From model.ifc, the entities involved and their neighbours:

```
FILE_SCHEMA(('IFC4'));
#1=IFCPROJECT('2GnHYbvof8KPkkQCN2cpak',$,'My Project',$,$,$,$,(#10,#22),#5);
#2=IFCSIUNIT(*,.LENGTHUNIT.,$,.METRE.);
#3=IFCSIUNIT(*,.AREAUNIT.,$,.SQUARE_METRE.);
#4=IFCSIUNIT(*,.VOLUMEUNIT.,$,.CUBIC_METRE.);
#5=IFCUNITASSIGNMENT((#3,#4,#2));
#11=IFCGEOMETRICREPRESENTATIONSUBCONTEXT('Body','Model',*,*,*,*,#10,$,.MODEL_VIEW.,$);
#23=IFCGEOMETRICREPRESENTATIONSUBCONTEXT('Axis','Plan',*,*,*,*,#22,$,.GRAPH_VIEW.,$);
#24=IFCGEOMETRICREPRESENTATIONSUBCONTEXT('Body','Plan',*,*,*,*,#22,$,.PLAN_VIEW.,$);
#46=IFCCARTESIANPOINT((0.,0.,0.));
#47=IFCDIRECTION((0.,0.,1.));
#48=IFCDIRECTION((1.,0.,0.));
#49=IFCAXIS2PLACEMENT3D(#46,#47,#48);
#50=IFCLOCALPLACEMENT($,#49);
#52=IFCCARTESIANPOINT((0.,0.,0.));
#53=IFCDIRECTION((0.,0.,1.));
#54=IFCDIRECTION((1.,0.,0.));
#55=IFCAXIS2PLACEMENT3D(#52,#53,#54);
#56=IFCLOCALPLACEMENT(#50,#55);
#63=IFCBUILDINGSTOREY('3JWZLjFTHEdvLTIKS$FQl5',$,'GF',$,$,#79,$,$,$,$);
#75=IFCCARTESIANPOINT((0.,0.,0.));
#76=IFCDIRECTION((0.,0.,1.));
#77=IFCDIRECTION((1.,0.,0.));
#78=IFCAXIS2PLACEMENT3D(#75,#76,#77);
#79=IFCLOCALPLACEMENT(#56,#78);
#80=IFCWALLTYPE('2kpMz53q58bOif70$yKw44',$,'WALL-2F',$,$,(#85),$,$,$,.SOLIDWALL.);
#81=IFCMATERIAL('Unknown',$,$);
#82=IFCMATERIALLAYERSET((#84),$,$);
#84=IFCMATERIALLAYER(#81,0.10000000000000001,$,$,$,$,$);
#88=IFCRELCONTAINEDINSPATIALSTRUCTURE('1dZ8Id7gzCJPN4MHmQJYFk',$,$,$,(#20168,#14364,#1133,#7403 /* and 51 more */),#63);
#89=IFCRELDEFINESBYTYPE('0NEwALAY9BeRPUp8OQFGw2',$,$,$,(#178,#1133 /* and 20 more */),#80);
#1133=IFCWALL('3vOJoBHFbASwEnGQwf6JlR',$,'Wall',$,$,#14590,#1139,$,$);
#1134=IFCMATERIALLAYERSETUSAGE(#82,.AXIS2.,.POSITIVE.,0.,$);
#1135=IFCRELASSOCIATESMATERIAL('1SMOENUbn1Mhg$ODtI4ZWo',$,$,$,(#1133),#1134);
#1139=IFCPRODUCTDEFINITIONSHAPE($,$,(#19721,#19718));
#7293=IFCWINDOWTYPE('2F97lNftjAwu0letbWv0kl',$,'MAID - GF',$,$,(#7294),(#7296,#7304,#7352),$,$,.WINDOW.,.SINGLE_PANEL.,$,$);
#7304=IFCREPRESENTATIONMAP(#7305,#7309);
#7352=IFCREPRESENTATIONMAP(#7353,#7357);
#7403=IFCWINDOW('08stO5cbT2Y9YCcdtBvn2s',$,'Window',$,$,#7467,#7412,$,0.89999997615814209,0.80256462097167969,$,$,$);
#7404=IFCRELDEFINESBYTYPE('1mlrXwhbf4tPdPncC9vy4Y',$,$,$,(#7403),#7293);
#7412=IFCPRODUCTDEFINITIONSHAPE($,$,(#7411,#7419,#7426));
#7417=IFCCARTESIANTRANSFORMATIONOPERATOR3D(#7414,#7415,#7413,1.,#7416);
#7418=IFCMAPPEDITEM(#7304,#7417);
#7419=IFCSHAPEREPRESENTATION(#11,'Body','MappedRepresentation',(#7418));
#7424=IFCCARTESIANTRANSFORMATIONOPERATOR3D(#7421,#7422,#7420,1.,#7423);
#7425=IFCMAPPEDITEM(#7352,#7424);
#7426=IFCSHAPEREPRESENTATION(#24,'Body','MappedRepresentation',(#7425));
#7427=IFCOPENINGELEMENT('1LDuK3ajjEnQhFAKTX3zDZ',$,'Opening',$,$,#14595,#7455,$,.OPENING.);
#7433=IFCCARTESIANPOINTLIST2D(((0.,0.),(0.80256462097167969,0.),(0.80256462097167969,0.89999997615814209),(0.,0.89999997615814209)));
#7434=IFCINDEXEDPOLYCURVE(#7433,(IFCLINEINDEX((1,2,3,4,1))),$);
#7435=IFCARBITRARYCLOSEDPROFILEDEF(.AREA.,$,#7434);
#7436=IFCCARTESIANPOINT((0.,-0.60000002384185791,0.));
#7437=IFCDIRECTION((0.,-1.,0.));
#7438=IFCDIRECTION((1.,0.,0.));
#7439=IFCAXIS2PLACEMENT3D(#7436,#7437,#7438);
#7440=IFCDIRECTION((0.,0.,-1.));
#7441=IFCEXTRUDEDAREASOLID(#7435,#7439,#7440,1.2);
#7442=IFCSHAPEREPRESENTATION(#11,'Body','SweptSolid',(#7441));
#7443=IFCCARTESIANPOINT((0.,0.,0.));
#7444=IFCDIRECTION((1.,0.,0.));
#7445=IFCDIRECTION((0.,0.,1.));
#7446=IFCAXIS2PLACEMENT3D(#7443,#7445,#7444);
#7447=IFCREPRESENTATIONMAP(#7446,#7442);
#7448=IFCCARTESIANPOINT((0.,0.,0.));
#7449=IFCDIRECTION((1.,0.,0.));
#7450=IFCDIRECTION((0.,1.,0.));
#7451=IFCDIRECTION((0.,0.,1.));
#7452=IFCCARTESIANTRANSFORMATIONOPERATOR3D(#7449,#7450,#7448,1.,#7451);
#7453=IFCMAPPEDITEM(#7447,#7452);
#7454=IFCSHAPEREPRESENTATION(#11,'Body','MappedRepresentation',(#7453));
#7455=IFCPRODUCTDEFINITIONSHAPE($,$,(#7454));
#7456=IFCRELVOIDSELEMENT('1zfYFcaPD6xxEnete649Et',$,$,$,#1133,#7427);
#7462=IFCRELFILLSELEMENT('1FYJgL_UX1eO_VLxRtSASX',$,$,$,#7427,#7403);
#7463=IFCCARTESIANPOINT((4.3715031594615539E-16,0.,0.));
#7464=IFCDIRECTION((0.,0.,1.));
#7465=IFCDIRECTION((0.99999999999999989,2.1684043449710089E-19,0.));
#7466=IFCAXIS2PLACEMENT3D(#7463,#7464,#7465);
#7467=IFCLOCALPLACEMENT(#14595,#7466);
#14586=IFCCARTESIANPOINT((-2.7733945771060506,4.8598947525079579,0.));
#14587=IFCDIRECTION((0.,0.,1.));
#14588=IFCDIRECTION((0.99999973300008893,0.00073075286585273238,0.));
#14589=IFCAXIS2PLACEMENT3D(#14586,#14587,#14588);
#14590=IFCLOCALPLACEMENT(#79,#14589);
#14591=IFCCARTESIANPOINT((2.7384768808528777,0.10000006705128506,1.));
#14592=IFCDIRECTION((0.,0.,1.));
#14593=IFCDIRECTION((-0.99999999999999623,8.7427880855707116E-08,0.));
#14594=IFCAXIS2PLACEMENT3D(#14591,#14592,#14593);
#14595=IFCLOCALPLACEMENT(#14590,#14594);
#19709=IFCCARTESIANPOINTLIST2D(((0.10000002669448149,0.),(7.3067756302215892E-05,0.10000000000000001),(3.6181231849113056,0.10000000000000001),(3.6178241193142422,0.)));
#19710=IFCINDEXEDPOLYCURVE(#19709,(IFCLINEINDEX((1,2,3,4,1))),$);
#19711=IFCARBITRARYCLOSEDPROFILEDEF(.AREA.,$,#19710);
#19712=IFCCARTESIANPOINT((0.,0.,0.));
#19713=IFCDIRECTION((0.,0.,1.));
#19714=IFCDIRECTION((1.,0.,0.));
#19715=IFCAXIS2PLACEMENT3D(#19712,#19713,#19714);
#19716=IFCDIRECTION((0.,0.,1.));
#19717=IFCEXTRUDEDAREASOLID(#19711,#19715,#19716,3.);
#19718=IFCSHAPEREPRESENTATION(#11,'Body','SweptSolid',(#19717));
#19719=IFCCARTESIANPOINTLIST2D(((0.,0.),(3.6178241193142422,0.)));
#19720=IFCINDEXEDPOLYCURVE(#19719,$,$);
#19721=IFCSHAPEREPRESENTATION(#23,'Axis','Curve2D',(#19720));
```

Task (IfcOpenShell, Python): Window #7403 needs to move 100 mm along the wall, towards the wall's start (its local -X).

```python
import ifcopenshell
import ifcopenshell.api.geometry
import ifcopenshell.util.placement

model = ifcopenshell.open("model.ifc")

window = model.by_guid("08stO5cbT2Y9YCcdtBvn2s")
opening = window.FillsVoids[0].RelatingOpeningElement
wall = opening.VoidsElements[0].RelatingBuildingElement

wall_matrix = ifcopenshell.util.placement.get_local_placement(wall.ObjectPlacement)
shift = wall_matrix[:3, 0] * -0.1
before = ifcopenshell.util.placement.get_local_placement(window.ObjectPlacement)[:3, 3].copy()

# The window is placed relative to its opening, so it follows when the opening moves.
matrix = ifcopenshell.util.placement.get_local_placement(opening.ObjectPlacement)
matrix[:3, 3] += shift
ifcopenshell.api.geometry.edit_object_placement(
    model, product=opening, matrix=matrix, is_si=False, should_transform_children=True
)

after = ifcopenshell.util.placement.get_local_placement(window.ObjectPlacement)[:3, 3]
print("window moved by", (after - before).round(3) + 0.0)

model.write("model_v2.ifc")
```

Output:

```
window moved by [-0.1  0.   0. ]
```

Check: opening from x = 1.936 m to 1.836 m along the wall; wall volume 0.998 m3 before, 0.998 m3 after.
